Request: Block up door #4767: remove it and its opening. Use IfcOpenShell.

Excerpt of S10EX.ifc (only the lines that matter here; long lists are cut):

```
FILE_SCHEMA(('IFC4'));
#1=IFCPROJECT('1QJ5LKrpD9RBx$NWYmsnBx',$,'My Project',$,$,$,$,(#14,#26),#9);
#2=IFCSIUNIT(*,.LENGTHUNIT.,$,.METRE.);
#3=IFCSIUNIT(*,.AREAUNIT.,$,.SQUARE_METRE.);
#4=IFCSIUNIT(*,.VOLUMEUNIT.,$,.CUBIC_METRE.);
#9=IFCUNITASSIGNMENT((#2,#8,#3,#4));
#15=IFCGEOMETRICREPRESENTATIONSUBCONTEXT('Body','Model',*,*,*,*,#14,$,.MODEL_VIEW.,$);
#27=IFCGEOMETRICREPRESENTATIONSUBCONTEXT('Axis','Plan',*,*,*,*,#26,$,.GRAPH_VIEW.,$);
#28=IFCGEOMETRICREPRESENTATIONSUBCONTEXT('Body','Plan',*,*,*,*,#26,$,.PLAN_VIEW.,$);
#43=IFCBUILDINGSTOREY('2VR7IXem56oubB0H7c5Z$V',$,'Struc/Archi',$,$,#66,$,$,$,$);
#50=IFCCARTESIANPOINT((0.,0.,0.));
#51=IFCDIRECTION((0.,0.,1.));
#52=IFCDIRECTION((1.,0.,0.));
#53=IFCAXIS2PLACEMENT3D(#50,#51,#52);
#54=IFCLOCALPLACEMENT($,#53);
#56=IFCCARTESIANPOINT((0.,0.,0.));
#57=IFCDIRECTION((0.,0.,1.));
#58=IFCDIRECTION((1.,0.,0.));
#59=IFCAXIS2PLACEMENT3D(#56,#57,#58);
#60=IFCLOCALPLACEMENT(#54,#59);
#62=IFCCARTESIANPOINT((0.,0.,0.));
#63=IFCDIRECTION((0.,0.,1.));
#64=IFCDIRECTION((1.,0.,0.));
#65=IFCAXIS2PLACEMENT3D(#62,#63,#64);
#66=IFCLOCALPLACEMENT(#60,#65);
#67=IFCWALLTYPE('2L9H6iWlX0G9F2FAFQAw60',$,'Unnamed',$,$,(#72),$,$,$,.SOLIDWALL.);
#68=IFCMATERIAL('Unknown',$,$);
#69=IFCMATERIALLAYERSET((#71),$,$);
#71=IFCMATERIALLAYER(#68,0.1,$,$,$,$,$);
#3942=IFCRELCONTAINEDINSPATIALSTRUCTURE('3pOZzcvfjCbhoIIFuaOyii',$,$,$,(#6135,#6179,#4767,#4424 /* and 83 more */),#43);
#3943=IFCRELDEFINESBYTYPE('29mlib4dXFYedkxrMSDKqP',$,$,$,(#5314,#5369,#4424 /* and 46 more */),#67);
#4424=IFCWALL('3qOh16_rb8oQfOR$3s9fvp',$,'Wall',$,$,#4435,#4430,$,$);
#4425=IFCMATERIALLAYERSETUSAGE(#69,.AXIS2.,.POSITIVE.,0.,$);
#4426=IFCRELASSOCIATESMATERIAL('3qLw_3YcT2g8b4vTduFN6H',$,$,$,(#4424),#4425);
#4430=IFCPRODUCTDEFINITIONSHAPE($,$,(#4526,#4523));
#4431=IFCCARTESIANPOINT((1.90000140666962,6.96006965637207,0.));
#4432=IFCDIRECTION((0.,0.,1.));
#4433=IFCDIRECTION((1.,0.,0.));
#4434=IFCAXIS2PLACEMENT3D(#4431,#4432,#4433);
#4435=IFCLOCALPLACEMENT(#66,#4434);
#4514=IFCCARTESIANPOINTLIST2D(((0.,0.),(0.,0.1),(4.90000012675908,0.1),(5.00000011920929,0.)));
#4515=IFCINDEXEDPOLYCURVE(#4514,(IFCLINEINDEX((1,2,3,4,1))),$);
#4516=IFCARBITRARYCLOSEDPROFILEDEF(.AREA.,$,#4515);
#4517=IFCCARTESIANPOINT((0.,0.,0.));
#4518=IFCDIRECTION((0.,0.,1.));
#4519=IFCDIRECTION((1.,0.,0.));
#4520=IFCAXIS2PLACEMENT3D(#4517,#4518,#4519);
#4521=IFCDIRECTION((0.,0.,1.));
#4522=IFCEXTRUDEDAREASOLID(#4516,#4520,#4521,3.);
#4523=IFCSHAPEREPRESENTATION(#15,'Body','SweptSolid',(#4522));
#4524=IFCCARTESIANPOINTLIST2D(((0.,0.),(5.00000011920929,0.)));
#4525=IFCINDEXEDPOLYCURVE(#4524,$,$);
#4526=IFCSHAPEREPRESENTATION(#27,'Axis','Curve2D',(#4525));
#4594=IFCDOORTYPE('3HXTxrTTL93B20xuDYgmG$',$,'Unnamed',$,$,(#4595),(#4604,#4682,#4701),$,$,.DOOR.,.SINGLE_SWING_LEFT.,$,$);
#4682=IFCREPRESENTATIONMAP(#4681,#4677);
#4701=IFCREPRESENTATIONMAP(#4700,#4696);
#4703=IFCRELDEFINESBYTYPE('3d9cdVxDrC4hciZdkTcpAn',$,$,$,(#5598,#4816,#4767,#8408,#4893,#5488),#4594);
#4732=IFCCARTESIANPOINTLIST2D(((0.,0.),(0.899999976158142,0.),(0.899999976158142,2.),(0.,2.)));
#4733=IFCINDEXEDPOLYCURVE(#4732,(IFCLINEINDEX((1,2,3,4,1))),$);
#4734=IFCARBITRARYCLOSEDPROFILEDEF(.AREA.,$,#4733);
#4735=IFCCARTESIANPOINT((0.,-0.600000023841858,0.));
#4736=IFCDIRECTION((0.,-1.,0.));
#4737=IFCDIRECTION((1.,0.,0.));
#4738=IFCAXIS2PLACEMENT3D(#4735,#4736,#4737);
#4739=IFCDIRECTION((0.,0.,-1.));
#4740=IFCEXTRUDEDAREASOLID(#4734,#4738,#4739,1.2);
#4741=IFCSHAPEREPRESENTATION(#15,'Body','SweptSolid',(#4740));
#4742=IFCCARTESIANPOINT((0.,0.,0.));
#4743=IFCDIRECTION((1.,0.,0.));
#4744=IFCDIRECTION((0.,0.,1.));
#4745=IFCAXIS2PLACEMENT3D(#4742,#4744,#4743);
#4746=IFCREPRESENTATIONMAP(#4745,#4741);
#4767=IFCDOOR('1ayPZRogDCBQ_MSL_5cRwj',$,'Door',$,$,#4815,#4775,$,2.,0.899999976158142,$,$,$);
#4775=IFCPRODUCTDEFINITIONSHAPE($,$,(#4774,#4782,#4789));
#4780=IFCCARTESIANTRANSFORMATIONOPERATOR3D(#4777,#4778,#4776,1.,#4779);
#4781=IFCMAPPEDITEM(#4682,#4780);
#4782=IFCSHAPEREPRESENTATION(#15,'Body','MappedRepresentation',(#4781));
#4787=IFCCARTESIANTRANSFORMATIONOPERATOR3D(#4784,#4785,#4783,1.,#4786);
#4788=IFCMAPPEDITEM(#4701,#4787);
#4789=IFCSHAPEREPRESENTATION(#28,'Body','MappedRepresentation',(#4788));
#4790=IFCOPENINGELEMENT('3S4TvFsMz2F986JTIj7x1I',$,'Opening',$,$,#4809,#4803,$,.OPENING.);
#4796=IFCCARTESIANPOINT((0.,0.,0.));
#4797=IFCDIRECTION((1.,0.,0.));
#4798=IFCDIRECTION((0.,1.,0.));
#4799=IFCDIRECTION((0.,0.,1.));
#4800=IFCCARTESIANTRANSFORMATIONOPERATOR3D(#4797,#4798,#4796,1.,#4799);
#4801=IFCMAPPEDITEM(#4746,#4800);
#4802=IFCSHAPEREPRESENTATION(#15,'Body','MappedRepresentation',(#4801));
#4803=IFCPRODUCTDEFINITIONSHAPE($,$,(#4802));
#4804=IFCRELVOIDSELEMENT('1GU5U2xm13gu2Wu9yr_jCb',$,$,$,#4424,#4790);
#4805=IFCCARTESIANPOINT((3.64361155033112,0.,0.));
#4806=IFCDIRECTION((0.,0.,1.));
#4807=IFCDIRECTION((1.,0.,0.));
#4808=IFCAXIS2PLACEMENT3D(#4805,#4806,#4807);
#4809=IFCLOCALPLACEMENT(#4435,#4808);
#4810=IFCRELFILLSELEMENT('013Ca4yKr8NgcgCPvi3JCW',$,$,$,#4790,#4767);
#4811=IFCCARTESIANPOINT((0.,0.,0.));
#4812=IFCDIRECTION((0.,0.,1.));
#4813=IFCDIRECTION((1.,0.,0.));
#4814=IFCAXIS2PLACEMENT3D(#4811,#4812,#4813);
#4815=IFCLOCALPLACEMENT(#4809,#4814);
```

```python
import ifcopenshell
import ifcopenshell.api.feature
import ifcopenshell.api.root
import ifcopenshell.geom
import ifcopenshell.util.shape

model = ifcopenshell.open("S10EX.ifc")
settings = ifcopenshell.geom.settings()


def volume(element):
    """Net volume in cubic metres, openings subtracted."""
    shape = ifcopenshell.geom.create_shape(settings, element)
    return ifcopenshell.util.shape.get_volume(shape.geometry)


door = model.by_guid("1ayPZRogDCBQ_MSL_5cRwj")
opening = door.FillsVoids[0].RelatingOpeningElement
wall = opening.VoidsElements[0].RelatingBuildingElement
before = volume(wall)

ifcopenshell.api.root.remove_product(model, product=door)
ifcopenshell.api.feature.remove_feature(model, feature=opening)

after = volume(wall)

print(f"wall volume {before:.3f} -> {after:.3f} m3")

model.write("S10EX_edited.ifc")
```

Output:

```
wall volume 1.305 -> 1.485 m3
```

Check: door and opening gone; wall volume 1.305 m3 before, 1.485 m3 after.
